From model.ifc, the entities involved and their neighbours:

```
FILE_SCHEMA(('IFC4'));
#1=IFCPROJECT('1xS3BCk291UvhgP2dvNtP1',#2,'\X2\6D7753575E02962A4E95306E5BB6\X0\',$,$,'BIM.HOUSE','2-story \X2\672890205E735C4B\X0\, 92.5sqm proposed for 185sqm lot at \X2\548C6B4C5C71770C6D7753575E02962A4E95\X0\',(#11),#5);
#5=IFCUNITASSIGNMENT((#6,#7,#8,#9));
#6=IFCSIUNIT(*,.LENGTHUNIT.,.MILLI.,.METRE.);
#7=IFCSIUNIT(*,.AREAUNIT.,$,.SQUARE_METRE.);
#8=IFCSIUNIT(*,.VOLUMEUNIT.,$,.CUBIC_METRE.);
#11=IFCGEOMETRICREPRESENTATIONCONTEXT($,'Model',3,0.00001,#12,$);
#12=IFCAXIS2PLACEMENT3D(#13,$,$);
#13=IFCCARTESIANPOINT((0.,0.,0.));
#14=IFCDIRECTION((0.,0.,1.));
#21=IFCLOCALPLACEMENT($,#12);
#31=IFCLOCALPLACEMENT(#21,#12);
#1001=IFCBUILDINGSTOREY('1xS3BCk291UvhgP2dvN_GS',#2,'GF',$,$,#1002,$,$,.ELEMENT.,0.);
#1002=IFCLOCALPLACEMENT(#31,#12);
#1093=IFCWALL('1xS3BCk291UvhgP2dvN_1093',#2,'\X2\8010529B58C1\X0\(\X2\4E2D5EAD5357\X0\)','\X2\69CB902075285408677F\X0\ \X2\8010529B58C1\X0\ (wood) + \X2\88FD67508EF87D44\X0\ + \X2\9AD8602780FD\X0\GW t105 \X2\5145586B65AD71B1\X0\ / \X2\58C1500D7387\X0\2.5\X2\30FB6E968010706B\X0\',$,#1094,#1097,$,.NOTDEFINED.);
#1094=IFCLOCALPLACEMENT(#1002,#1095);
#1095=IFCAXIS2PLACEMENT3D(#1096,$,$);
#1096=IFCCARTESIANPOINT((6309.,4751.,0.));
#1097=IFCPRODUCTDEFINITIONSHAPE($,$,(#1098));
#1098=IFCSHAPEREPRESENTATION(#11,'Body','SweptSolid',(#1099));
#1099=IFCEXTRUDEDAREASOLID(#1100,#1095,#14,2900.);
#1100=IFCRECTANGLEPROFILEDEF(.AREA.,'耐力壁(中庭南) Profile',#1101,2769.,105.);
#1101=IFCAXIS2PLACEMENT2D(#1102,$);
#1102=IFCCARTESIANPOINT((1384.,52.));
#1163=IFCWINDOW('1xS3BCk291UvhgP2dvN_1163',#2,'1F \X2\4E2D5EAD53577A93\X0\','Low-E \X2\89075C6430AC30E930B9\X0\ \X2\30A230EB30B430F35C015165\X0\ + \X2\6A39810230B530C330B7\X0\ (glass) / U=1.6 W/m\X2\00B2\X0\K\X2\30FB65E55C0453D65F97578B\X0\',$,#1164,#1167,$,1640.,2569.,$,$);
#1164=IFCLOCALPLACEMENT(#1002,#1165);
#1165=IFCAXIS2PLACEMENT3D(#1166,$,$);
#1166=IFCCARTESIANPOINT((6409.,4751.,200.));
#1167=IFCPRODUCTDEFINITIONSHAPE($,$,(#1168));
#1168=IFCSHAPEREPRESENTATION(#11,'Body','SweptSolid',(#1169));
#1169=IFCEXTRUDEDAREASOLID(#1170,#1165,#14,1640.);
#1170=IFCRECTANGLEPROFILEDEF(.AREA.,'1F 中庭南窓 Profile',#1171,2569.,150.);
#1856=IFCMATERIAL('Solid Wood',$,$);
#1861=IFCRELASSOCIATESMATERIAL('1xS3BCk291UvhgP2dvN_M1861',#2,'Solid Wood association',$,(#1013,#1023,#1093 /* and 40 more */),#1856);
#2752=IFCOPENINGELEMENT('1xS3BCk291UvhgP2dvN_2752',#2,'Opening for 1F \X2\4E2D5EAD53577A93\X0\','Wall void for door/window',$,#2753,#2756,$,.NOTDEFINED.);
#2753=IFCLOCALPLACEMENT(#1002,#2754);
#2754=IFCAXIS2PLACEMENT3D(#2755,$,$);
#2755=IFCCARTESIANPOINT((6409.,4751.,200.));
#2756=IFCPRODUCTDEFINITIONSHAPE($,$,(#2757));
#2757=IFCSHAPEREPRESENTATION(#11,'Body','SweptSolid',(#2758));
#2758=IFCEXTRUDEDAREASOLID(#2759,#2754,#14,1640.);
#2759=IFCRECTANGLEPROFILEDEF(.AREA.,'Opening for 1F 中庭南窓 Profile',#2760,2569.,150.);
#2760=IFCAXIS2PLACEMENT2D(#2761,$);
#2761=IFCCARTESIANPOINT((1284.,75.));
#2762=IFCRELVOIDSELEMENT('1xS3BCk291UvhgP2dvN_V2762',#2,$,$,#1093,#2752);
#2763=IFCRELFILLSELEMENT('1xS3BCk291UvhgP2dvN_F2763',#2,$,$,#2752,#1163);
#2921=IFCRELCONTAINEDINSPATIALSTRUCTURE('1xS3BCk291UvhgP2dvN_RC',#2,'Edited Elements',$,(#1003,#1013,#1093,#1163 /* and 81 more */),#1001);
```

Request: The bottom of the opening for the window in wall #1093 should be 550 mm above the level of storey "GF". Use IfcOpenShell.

```python
import numpy as np
import ifcopenshell
import ifcopenshell.api.geometry
import ifcopenshell.geom
import ifcopenshell.util.element
import ifcopenshell.util.placement
import ifcopenshell.util.shape
import ifcopenshell.util.unit

model = ifcopenshell.open("model.ifc")
unit_scale = ifcopenshell.util.unit.calculate_unit_scale(model)

window = model.by_guid("1xS3BCk291UvhgP2dvN_1163")
opening = window.FillsVoids[0].RelatingOpeningElement
storey = ifcopenshell.util.element.get_container(window, ifc_class="IfcBuildingStorey")
level = ifcopenshell.util.placement.get_local_placement(storey.ObjectPlacement)[2, 3]

# The opening's origin need not be at the sill, so measure its lowest point.
shape = ifcopenshell.geom.create_shape(ifcopenshell.geom.settings(), opening)
bottom = ifcopenshell.util.shape.get_shape_bottom_elevation(shape, shape.geometry) / unit_scale
dz = level + 0.55 / unit_scale - bottom

shift = np.array([0.0, 0.0, dz])
# The window is not placed relative to its opening, so move both.
for product in (opening, window):
    matrix = ifcopenshell.util.placement.get_local_placement(product.ObjectPlacement)
    matrix[:3, 3] += shift
    ifcopenshell.api.geometry.edit_object_placement(model, product=product, matrix=matrix, is_si=False)

print(f"moved by {dz * unit_scale:+.3f} m")

model.write("model_rev.ifc")
```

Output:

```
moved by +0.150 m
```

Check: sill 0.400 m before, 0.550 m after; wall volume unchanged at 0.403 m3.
